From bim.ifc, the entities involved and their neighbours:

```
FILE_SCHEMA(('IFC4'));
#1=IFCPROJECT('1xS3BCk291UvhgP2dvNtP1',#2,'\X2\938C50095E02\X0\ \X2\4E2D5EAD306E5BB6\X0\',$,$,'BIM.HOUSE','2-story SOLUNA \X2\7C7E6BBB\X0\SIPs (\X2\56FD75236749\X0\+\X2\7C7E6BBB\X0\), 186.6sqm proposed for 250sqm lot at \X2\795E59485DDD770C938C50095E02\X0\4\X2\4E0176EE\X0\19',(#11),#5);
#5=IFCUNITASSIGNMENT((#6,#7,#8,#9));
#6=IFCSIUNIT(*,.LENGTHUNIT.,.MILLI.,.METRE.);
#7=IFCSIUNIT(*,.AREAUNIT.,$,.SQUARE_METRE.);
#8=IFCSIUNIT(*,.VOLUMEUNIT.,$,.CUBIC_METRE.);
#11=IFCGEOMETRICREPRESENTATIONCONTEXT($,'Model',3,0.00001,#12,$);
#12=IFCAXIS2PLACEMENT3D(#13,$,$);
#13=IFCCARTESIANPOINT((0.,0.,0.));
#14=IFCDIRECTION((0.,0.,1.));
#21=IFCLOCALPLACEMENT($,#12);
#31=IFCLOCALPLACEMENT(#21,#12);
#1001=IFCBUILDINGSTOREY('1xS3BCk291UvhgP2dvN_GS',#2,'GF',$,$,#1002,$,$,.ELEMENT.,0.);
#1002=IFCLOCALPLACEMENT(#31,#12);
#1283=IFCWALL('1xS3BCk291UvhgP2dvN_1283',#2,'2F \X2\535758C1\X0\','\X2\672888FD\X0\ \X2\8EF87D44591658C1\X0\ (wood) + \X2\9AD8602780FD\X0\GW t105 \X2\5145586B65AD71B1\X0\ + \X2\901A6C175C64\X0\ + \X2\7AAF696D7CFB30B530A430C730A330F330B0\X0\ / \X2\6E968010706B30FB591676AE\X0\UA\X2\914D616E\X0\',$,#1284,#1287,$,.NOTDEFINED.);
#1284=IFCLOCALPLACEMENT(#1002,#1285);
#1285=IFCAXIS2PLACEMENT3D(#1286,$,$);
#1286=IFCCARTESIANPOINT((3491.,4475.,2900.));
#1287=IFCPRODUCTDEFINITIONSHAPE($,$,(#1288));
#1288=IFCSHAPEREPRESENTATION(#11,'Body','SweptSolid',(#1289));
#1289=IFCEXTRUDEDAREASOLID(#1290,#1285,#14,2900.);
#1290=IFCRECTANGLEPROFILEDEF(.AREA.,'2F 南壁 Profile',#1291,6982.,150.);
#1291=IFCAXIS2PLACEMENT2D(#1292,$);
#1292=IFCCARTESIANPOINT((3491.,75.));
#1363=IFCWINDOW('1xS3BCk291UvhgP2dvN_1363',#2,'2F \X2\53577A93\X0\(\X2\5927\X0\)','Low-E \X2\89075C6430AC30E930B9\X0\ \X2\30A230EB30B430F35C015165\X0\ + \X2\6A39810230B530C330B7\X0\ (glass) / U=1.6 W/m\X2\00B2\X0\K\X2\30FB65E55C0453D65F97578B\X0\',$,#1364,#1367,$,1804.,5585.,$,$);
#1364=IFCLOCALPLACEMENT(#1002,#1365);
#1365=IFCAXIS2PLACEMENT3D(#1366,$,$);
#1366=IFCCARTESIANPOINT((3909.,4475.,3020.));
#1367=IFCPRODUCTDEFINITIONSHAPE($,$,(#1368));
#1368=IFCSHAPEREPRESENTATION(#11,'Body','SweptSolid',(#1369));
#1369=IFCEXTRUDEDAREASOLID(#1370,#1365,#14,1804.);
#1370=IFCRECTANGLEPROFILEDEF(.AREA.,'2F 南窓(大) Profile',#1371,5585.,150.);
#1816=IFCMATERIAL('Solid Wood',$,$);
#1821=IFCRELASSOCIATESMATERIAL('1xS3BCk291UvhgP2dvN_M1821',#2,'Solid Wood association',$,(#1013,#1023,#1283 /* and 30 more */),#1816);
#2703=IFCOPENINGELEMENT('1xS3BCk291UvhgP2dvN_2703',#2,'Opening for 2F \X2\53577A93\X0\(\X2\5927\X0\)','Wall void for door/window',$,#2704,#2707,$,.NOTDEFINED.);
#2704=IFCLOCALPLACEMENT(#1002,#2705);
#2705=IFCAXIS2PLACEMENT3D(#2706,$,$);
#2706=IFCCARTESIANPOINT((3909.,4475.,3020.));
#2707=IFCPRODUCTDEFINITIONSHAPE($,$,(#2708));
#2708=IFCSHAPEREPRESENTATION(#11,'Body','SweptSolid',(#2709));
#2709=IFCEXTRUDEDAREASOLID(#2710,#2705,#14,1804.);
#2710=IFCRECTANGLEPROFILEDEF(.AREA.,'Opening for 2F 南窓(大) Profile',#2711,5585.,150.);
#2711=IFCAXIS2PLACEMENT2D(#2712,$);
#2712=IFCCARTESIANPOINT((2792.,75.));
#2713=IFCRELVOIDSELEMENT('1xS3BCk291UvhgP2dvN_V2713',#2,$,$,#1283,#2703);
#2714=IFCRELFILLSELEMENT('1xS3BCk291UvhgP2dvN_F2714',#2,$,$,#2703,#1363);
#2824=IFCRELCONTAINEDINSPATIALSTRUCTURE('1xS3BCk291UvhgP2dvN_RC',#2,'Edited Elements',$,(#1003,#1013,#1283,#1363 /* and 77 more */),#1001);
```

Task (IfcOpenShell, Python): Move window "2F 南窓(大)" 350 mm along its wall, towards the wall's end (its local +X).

```python
import ifcopenshell
import ifcopenshell.api.geometry
import ifcopenshell.util.placement

model = ifcopenshell.open("bim.ifc")

window = model.by_guid("1xS3BCk291UvhgP2dvN_1363")
opening = window.FillsVoids[0].RelatingOpeningElement
wall = opening.VoidsElements[0].RelatingBuildingElement

wall_matrix = ifcopenshell.util.placement.get_local_placement(wall.ObjectPlacement)
shift = wall_matrix[:3, 0] * 350.0
before = ifcopenshell.util.placement.get_local_placement(window.ObjectPlacement)[:3, 3].copy()

# The window is not placed relative to its opening, so move both.
for product in (opening, window):
    matrix = ifcopenshell.util.placement.get_local_placement(product.ObjectPlacement)
    matrix[:3, 3] += shift
    ifcopenshell.api.geometry.edit_object_placement(model, product=product, matrix=matrix, is_si=False)

after = ifcopenshell.util.placement.get_local_placement(window.ObjectPlacement)[:3, 3]
print("window moved by", (after - before).round(3) + 0.0)

model.write("bim-out.ifc")
```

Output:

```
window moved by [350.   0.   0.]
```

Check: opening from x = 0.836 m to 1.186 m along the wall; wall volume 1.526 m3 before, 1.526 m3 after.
